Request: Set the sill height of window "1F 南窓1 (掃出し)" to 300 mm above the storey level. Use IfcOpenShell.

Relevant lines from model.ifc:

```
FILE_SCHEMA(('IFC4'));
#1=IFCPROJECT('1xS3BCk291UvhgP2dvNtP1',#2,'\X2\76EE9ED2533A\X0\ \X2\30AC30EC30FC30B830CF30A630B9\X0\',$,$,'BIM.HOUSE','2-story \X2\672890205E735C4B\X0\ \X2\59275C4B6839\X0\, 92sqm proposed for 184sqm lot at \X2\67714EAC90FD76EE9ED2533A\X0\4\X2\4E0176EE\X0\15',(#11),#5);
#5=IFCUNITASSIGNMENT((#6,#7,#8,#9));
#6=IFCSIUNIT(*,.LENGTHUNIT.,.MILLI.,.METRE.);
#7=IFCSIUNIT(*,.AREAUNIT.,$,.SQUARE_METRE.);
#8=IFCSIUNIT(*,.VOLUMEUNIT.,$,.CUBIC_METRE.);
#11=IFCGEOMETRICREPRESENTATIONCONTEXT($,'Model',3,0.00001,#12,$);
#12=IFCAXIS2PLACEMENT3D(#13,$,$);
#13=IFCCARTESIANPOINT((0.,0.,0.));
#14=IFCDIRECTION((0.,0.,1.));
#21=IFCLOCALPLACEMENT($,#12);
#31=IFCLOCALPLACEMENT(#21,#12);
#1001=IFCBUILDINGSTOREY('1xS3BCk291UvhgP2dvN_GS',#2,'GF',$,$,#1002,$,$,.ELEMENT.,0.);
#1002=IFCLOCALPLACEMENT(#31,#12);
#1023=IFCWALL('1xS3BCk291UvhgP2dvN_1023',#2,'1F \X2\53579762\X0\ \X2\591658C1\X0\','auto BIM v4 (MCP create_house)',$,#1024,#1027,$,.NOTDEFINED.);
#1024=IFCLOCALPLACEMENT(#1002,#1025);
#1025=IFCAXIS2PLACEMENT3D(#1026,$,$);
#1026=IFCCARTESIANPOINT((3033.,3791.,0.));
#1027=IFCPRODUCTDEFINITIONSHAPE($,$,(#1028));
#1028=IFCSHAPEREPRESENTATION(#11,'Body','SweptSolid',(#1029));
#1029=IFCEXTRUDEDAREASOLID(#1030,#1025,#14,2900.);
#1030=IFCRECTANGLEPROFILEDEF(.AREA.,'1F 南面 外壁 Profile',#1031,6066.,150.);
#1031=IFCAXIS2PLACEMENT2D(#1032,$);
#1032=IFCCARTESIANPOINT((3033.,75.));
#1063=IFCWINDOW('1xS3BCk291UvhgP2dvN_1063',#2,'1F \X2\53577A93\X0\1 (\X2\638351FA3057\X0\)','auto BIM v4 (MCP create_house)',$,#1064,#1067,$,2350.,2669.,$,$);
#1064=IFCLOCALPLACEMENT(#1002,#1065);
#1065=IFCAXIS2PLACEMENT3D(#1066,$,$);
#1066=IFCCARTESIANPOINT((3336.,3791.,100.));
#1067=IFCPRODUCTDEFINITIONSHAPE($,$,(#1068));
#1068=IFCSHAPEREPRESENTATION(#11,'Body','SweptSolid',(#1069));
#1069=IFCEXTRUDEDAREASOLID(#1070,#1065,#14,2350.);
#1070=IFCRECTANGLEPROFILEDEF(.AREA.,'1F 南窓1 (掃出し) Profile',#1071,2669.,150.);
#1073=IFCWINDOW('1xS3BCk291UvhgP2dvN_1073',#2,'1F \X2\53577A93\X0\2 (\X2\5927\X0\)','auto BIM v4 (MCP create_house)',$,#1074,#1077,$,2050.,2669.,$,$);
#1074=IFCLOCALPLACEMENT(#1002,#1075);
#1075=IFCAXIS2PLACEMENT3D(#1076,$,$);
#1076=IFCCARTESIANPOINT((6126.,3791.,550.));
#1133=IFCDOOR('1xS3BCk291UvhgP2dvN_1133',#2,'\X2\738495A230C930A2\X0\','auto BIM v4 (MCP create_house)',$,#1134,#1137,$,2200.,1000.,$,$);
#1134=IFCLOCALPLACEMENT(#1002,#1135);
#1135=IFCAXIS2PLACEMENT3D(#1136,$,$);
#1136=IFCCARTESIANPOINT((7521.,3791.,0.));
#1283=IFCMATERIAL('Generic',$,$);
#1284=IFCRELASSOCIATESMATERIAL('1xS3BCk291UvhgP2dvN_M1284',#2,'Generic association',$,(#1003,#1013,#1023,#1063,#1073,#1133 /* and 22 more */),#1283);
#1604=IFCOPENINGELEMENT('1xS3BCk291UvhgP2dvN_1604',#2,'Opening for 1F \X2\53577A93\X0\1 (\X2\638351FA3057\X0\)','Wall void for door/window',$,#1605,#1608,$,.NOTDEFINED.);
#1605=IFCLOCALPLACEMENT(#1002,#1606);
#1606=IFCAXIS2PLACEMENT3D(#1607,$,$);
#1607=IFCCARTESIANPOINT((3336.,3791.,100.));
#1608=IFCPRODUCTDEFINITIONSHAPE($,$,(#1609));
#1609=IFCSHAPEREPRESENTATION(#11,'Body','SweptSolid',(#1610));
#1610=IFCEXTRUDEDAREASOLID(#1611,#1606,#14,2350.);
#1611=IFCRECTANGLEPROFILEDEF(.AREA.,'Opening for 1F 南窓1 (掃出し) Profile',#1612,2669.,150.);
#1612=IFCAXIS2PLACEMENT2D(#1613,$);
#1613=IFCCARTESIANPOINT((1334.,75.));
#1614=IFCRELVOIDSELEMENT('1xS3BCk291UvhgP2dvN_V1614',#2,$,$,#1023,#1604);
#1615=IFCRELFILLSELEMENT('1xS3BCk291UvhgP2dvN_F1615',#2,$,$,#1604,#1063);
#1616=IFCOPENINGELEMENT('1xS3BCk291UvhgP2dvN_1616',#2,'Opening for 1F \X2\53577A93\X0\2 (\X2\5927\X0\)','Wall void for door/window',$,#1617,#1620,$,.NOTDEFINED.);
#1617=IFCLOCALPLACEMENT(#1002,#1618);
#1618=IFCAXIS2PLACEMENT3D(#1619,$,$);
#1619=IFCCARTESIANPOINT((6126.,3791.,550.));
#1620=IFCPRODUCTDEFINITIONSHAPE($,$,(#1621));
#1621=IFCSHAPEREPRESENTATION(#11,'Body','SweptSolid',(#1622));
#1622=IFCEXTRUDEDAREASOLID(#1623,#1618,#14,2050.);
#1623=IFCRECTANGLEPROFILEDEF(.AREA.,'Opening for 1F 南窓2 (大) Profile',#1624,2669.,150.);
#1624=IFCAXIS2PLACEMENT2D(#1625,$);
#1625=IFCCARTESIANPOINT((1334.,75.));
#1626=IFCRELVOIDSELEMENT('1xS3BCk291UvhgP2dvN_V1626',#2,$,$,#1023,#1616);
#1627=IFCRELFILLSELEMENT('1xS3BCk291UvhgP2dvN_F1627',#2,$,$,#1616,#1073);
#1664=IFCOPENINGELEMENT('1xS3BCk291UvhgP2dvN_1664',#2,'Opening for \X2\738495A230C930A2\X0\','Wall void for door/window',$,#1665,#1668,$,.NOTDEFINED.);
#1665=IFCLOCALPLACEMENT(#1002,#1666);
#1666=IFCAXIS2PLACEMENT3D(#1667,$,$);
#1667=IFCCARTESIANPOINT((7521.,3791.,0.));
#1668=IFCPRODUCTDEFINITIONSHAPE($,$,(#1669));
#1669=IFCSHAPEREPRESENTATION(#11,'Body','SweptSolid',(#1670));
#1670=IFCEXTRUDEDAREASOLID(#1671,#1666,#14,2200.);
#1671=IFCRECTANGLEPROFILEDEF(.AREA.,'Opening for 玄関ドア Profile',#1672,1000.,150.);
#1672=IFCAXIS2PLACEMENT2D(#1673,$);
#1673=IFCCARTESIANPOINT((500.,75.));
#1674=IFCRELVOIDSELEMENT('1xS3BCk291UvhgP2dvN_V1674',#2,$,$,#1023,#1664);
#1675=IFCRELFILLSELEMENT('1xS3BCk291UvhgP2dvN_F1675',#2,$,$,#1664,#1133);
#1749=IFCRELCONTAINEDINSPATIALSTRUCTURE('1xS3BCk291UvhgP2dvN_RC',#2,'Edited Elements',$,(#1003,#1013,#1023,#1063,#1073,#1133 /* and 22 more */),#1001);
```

```python
import numpy as np
import ifcopenshell
import ifcopenshell.api.geometry
import ifcopenshell.geom
import ifcopenshell.util.element
import ifcopenshell.util.placement
import ifcopenshell.util.shape
import ifcopenshell.util.unit

model = ifcopenshell.open("model.ifc")
unit_scale = ifcopenshell.util.unit.calculate_unit_scale(model)

window = model.by_id(1063)
opening = window.FillsVoids[0].RelatingOpeningElement
storey = ifcopenshell.util.element.get_container(window, ifc_class="IfcBuildingStorey")
level = ifcopenshell.util.placement.get_local_placement(storey.ObjectPlacement)[2, 3]

# The opening's origin need not be at the sill, so measure its lowest point.
shape = ifcopenshell.geom.create_shape(ifcopenshell.geom.settings(), opening)
bottom = ifcopenshell.util.shape.get_shape_bottom_elevation(shape, shape.geometry) / unit_scale
dz = level + 0.3 / unit_scale - bottom

shift = np.array([0.0, 0.0, dz])
# The window is not placed relative to its opening, so move both.
for product in (opening, window):
    matrix = ifcopenshell.util.placement.get_local_placement(product.ObjectPlacement)
    matrix[:3, 3] += shift
    ifcopenshell.api.geometry.edit_object_placement(model, product=product, matrix=matrix, is_si=False)

print(f"moved by {dz * unit_scale:+.3f} m")

model.write("model_rev.ifc")
```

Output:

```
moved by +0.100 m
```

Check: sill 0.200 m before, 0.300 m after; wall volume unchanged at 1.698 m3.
